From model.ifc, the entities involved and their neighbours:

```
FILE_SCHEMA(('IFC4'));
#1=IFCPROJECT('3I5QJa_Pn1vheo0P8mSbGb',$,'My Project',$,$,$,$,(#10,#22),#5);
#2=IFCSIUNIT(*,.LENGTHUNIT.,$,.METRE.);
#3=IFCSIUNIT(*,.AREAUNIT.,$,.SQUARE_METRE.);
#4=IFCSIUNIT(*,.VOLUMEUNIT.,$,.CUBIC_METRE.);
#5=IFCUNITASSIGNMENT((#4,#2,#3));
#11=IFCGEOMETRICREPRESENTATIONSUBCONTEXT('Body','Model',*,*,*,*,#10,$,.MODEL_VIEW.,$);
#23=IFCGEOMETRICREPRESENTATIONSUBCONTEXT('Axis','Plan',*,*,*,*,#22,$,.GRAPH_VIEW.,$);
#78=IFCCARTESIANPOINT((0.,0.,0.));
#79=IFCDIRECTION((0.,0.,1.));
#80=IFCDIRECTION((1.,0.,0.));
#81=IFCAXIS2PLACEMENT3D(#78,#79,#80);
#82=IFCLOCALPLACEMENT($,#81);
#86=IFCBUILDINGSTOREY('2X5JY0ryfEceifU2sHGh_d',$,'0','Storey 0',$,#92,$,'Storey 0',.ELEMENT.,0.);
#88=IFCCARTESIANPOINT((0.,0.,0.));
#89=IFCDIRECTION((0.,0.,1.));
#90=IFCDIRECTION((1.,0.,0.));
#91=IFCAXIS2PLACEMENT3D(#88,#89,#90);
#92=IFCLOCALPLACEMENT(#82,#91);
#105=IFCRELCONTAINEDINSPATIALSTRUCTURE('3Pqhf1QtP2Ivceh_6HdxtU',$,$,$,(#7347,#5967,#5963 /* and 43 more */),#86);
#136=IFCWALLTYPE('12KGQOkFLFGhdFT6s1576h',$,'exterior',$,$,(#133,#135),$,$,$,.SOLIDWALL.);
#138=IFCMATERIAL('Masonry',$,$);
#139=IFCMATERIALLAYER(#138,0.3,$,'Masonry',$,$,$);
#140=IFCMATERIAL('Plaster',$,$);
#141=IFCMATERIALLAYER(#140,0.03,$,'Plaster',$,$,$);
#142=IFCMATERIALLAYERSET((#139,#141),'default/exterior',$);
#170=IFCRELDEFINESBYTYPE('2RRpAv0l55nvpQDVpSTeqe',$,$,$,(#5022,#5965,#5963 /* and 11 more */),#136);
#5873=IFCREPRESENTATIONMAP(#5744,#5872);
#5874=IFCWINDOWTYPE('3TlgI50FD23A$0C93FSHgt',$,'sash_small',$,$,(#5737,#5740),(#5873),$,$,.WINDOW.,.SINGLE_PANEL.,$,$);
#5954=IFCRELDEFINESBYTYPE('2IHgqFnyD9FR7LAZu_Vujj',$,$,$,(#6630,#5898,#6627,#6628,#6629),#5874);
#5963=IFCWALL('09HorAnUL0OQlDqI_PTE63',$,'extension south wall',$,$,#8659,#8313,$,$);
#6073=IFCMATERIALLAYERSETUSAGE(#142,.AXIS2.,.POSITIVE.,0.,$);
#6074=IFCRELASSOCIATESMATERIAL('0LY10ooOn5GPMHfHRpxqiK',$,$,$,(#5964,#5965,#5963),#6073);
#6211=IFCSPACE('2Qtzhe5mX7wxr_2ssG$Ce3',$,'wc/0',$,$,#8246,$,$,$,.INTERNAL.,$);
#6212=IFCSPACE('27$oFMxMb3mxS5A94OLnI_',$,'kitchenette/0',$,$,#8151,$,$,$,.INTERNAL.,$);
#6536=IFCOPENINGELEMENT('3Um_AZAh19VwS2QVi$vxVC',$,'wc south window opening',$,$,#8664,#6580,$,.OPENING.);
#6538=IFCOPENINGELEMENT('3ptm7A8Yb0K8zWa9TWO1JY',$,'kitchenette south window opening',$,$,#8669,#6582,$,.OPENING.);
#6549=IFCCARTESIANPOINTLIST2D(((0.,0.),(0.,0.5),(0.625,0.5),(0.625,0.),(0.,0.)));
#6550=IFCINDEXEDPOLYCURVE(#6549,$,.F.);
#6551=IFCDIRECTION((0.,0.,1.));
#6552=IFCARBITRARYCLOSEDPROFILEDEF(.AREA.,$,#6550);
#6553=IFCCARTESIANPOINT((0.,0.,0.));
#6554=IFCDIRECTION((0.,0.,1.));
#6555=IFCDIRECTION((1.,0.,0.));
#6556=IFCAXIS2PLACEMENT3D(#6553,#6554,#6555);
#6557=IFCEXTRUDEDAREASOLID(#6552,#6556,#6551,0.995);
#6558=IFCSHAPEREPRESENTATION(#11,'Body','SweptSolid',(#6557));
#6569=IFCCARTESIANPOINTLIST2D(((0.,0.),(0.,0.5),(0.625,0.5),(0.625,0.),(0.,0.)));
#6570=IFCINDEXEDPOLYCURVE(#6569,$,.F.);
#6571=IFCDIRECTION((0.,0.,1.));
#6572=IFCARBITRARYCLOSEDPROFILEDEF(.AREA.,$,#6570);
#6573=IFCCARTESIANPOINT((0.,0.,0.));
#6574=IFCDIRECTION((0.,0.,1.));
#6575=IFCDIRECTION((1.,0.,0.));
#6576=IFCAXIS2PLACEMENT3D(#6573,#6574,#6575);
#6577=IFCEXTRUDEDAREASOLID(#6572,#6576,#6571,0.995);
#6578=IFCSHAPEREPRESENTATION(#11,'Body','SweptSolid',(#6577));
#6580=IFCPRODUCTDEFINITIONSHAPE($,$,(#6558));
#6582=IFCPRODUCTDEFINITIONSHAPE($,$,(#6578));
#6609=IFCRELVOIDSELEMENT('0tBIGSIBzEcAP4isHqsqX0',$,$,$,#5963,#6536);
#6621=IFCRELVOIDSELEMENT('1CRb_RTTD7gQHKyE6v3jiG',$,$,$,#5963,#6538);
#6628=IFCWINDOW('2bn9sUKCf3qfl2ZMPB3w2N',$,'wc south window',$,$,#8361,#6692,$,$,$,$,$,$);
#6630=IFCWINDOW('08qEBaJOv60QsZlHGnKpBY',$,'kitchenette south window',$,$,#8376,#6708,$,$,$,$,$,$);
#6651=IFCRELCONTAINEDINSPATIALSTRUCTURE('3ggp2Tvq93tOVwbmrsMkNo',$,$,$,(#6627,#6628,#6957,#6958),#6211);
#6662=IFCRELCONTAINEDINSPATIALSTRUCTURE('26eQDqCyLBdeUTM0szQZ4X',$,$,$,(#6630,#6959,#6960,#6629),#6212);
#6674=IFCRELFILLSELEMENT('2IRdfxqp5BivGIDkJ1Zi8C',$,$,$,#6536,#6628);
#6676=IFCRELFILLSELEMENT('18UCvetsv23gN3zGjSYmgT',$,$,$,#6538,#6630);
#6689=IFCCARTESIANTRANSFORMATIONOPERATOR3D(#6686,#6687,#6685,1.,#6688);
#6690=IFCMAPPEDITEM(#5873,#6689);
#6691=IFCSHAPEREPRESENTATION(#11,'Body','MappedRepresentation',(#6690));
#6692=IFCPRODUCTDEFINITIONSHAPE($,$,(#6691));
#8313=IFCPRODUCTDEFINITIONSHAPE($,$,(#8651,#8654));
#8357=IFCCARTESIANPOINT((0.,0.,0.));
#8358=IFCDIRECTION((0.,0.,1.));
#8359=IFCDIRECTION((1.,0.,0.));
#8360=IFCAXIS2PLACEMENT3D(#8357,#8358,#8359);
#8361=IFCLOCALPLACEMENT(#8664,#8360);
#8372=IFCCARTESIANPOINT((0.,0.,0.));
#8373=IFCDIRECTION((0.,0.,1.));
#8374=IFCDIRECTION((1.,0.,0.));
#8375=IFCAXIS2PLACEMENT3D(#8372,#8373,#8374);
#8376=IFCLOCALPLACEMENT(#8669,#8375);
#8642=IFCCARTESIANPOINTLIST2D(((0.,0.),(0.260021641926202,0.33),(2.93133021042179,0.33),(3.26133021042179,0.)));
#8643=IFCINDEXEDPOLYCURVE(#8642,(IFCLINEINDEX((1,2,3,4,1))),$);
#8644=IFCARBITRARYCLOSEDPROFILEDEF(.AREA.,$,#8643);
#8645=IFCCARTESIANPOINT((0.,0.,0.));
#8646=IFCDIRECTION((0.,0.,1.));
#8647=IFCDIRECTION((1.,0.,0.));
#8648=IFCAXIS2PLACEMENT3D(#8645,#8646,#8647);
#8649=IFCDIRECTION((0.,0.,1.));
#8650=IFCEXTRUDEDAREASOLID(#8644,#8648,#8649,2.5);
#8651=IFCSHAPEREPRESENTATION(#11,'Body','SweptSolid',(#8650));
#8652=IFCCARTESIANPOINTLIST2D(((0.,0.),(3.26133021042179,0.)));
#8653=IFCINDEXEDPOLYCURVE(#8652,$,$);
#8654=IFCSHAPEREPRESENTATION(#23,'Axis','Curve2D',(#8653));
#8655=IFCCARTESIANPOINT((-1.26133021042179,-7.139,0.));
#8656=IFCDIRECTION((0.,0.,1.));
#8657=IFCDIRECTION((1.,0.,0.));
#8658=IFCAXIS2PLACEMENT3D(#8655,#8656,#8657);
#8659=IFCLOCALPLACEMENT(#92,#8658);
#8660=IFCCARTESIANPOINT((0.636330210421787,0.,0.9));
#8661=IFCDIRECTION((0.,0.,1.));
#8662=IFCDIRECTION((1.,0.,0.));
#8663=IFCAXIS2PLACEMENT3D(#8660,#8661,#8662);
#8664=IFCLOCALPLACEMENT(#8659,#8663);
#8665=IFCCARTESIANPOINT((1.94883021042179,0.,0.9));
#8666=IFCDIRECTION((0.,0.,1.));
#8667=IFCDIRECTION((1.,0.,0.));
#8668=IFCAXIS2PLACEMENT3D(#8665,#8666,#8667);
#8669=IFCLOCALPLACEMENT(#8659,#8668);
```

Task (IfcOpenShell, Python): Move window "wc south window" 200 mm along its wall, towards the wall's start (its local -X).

```python
import ifcopenshell
import ifcopenshell.api.geometry
import ifcopenshell.util.placement

model = ifcopenshell.open("model.ifc")

window = model.by_id(6628)
opening = window.FillsVoids[0].RelatingOpeningElement
wall = opening.VoidsElements[0].RelatingBuildingElement

wall_matrix = ifcopenshell.util.placement.get_local_placement(wall.ObjectPlacement)
shift = wall_matrix[:3, 0] * -0.2
before = ifcopenshell.util.placement.get_local_placement(window.ObjectPlacement)[:3, 3].copy()

# The window is placed relative to its opening, so it follows when the opening moves.
matrix = ifcopenshell.util.placement.get_local_placement(opening.ObjectPlacement)
matrix[:3, 3] += shift
ifcopenshell.api.geometry.edit_object_placement(
    model, product=opening, matrix=matrix, is_si=False, should_transform_children=True
)

after = ifcopenshell.util.placement.get_local_placement(window.ObjectPlacement)[:3, 3]
print("window moved by", (after - before).round(3) + 0.0)

model.write("model_edited.ifc")
```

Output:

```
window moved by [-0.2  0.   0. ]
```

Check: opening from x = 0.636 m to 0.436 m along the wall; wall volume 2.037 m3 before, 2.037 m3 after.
